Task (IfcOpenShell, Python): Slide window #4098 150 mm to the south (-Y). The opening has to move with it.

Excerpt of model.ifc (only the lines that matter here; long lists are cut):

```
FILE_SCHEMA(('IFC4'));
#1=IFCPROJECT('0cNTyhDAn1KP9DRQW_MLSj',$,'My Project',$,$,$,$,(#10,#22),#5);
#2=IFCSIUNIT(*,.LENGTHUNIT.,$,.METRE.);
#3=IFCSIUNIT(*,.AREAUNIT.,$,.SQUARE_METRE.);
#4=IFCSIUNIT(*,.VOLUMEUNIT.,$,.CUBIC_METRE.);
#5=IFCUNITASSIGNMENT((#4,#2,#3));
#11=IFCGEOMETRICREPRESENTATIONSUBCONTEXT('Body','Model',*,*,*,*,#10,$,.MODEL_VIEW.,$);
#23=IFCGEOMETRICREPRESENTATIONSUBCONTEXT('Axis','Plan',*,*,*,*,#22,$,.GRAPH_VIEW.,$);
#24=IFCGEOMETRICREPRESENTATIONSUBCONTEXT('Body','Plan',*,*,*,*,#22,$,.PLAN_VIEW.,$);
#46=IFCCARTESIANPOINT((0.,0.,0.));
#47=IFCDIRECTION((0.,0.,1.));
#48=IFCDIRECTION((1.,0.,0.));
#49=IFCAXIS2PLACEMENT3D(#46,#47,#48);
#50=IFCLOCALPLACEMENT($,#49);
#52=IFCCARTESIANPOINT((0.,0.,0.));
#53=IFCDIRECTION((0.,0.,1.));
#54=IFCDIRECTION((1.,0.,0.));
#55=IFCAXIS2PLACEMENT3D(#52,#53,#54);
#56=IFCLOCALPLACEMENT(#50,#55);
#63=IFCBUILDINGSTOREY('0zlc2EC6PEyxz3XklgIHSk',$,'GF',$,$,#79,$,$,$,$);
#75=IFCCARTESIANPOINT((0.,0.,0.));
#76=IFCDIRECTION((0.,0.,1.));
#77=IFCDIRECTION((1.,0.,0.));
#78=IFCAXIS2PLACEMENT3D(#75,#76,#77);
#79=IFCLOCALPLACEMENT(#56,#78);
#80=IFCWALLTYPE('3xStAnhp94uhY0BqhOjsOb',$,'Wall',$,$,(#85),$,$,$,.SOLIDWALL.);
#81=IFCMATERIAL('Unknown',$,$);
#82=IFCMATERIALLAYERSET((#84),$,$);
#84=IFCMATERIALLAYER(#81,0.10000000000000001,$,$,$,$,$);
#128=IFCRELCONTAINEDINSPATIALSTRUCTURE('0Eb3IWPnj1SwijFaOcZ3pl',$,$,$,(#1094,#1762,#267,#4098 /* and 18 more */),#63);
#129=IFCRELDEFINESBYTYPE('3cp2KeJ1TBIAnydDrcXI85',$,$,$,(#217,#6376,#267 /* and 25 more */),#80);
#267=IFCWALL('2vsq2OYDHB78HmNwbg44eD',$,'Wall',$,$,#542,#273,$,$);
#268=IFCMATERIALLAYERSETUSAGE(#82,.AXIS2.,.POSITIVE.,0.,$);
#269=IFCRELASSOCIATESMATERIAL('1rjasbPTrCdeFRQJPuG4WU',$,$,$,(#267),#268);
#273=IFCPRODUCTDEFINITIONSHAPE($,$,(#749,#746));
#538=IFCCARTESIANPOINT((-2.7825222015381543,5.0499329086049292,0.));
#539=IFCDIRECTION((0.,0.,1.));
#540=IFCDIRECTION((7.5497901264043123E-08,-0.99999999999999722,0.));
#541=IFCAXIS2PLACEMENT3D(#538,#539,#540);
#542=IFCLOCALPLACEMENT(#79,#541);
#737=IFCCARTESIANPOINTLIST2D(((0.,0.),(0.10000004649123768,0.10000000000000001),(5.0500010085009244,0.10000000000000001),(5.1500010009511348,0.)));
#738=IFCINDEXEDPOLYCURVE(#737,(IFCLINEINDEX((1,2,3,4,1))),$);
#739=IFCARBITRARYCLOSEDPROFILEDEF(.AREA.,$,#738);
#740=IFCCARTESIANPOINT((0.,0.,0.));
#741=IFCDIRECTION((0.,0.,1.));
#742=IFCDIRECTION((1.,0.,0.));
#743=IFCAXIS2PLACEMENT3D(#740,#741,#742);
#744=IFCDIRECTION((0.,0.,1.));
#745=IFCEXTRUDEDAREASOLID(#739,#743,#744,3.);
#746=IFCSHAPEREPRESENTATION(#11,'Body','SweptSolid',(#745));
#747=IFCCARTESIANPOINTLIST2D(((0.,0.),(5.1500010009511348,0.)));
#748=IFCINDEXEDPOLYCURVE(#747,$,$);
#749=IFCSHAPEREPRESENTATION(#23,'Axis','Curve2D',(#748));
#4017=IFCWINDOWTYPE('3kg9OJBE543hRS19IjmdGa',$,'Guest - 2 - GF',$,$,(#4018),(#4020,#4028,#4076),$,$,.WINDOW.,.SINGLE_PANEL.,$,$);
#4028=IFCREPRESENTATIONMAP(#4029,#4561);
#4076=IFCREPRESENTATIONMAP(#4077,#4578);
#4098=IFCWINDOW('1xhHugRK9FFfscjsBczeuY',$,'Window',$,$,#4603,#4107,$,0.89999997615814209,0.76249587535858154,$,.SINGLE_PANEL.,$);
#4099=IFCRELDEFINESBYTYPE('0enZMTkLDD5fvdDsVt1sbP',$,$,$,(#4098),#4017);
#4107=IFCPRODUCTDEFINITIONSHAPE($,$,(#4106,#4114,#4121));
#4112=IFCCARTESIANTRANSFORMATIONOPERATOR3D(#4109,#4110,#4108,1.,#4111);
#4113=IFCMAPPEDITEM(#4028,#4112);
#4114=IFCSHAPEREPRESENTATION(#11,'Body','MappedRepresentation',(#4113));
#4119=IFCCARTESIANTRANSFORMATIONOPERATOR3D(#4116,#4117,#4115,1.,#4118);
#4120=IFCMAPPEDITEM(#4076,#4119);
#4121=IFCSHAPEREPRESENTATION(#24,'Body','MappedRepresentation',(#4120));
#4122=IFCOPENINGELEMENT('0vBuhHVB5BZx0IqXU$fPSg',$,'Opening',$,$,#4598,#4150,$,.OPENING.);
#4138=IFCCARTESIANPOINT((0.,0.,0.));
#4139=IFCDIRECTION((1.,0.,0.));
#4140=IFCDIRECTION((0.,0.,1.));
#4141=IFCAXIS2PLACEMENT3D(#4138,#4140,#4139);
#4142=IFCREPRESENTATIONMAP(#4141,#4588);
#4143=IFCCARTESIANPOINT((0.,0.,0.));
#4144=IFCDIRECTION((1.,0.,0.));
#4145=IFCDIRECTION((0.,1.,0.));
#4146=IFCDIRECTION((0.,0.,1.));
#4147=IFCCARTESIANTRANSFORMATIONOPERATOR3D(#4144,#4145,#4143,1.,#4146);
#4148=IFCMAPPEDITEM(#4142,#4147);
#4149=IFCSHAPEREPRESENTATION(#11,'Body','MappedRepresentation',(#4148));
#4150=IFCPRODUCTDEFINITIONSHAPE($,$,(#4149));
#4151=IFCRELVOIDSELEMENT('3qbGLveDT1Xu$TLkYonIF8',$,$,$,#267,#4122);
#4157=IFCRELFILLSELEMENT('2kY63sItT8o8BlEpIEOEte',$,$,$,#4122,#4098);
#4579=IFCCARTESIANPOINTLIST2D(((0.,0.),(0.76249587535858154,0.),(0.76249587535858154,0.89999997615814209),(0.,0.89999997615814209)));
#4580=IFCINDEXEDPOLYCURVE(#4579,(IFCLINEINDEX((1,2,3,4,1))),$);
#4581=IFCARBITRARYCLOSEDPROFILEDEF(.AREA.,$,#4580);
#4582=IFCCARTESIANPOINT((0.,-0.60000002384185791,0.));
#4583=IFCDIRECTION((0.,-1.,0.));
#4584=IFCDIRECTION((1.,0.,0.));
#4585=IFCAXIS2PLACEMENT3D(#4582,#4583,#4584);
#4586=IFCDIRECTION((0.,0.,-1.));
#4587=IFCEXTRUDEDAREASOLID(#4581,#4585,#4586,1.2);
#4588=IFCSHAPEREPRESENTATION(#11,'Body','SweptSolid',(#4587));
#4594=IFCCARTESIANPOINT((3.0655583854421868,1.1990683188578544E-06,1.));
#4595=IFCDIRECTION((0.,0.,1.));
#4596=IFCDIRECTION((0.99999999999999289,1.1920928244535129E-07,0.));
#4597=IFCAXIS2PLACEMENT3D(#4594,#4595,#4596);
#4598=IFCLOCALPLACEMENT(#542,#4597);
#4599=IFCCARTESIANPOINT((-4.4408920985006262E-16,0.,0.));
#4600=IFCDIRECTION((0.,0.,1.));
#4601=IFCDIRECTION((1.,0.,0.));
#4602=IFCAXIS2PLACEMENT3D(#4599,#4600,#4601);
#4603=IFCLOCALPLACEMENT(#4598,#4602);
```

```python
import ifcopenshell
import ifcopenshell.api.geometry
import ifcopenshell.util.placement
import ifcopenshell.util.unit

model = ifcopenshell.open("model.ifc")
unit_scale = ifcopenshell.util.unit.calculate_unit_scale(model)

window = model.by_guid("1xhHugRK9FFfscjsBczeuY")
opening = window.FillsVoids[0].RelatingOpeningElement
wall = opening.VoidsElements[0].RelatingBuildingElement

wall_matrix = ifcopenshell.util.placement.get_local_placement(wall.ObjectPlacement)
shift = wall_matrix[:3, 0] * 0.15 / unit_scale
before = ifcopenshell.util.placement.get_local_placement(window.ObjectPlacement)[:3, 3].copy()

# The window is placed relative to its opening, so it follows when the opening moves.
matrix = ifcopenshell.util.placement.get_local_placement(opening.ObjectPlacement)
matrix[:3, 3] += shift
ifcopenshell.api.geometry.edit_object_placement(
    model, product=opening, matrix=matrix, is_si=False, should_transform_children=True
)

after = ifcopenshell.util.placement.get_local_placement(window.ObjectPlacement)[:3, 3]
print("window moved by", (after - before).round(3) + 0.0)

model.write("model_updated.ifc")
```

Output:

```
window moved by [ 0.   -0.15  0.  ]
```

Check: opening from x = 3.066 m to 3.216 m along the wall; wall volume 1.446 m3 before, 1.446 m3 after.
